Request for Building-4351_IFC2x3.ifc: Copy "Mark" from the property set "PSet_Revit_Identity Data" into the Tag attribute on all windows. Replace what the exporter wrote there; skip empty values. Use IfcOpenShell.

First a look at what the model holds.

```python
import ifcopenshell
import ifcopenshell.util.element

model = ifcopenshell.open("Building-4351_IFC2x3.ifc")
print(model.schema)
windows = model.by_type("IfcWindow")
print(len(windows), "windows")
for e in windows[:8]:
    source = ifcopenshell.util.element.get_pset(e, "PSet_Revit_Identity Data", "Mark")
    target = e.Tag
    print(e.id(), repr(source), repr(target), sep=" | ")
```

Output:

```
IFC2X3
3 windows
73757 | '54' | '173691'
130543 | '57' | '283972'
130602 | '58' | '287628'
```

```python
import ifcopenshell
import ifcopenshell.util.element

model = ifcopenshell.open("Building-4351_IFC2x3.ifc")

count = 0
for e in model.by_type("IfcWindow"):
    value = ifcopenshell.util.element.get_pset(e, "PSet_Revit_Identity Data", "Mark")
    current = e.Tag
    if not value or not value.strip() or current == value:
        continue
    e.Tag = value
    count += 1

print(count, "windows updated")

model.write("Building-4351_IFC2x3-out.ifc")
```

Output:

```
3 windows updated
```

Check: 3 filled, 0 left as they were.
